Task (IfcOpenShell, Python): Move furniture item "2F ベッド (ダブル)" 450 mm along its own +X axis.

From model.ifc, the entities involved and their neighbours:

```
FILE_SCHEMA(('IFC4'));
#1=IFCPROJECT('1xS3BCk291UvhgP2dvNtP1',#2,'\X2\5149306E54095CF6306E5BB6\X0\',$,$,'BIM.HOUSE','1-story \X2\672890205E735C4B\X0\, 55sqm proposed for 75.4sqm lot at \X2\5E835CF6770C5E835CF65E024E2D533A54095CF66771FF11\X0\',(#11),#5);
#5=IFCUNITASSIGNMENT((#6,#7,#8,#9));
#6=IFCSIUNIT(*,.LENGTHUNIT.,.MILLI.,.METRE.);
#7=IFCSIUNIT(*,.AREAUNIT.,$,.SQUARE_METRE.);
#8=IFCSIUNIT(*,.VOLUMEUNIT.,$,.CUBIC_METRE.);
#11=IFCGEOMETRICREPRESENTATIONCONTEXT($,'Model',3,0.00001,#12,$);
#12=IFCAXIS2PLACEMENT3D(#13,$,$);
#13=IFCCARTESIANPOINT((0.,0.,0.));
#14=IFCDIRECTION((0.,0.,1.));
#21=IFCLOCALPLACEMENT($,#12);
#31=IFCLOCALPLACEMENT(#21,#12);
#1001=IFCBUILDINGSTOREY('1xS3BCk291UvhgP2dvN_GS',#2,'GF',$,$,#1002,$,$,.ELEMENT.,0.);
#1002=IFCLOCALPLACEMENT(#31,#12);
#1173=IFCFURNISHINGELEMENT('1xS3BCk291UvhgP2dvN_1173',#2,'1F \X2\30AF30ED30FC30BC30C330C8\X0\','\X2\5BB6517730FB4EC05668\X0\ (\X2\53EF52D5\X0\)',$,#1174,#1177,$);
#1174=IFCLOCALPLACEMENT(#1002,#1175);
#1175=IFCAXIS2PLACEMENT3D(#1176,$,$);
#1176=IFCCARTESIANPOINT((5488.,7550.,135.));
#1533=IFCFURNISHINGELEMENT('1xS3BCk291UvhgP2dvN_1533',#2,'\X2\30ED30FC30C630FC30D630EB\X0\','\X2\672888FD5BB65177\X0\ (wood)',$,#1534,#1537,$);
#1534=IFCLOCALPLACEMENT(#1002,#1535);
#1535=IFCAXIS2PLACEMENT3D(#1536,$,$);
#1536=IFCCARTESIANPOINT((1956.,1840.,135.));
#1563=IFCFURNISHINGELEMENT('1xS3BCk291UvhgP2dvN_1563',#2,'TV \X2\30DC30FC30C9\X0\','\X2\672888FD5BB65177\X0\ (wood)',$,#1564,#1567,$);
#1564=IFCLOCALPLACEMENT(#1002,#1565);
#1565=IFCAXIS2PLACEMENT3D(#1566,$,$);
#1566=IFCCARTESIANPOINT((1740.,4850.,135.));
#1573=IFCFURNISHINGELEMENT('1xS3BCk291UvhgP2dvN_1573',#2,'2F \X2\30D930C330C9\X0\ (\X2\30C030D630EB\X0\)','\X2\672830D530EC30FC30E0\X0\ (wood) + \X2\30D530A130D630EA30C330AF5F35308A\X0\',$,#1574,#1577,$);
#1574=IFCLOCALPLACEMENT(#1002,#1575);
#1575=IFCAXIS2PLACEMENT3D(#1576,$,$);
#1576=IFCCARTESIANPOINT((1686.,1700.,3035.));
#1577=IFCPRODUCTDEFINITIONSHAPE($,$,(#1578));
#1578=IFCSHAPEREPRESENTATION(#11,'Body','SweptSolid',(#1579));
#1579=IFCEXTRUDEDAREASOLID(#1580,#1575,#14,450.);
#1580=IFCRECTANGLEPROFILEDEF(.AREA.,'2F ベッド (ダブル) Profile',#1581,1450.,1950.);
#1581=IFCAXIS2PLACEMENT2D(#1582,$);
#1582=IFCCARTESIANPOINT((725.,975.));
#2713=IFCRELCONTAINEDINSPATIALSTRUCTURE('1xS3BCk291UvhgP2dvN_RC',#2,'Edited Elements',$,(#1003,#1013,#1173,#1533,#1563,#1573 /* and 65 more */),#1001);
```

```python
import ifcopenshell
import ifcopenshell.api.geometry
import ifcopenshell.util.placement
import ifcopenshell.util.unit

model = ifcopenshell.open("model.ifc")
unit_scale = ifcopenshell.util.unit.calculate_unit_scale(model)

item = model.by_guid("1xS3BCk291UvhgP2dvN_1573")
matrix = ifcopenshell.util.placement.get_local_placement(item.ObjectPlacement)
matrix[:3, 3] += matrix[:3, 0] * 0.45 / unit_scale
ifcopenshell.api.geometry.edit_object_placement(model, product=item, matrix=matrix, is_si=False)

print(ifcopenshell.util.placement.get_local_placement(item.ObjectPlacement).round(3) + 0.0)

model.write("model_updated.ifc")
```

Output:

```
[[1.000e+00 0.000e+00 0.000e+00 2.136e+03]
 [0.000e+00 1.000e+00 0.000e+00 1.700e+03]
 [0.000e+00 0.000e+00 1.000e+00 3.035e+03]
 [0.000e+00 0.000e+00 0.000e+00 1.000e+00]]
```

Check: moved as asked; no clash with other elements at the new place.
